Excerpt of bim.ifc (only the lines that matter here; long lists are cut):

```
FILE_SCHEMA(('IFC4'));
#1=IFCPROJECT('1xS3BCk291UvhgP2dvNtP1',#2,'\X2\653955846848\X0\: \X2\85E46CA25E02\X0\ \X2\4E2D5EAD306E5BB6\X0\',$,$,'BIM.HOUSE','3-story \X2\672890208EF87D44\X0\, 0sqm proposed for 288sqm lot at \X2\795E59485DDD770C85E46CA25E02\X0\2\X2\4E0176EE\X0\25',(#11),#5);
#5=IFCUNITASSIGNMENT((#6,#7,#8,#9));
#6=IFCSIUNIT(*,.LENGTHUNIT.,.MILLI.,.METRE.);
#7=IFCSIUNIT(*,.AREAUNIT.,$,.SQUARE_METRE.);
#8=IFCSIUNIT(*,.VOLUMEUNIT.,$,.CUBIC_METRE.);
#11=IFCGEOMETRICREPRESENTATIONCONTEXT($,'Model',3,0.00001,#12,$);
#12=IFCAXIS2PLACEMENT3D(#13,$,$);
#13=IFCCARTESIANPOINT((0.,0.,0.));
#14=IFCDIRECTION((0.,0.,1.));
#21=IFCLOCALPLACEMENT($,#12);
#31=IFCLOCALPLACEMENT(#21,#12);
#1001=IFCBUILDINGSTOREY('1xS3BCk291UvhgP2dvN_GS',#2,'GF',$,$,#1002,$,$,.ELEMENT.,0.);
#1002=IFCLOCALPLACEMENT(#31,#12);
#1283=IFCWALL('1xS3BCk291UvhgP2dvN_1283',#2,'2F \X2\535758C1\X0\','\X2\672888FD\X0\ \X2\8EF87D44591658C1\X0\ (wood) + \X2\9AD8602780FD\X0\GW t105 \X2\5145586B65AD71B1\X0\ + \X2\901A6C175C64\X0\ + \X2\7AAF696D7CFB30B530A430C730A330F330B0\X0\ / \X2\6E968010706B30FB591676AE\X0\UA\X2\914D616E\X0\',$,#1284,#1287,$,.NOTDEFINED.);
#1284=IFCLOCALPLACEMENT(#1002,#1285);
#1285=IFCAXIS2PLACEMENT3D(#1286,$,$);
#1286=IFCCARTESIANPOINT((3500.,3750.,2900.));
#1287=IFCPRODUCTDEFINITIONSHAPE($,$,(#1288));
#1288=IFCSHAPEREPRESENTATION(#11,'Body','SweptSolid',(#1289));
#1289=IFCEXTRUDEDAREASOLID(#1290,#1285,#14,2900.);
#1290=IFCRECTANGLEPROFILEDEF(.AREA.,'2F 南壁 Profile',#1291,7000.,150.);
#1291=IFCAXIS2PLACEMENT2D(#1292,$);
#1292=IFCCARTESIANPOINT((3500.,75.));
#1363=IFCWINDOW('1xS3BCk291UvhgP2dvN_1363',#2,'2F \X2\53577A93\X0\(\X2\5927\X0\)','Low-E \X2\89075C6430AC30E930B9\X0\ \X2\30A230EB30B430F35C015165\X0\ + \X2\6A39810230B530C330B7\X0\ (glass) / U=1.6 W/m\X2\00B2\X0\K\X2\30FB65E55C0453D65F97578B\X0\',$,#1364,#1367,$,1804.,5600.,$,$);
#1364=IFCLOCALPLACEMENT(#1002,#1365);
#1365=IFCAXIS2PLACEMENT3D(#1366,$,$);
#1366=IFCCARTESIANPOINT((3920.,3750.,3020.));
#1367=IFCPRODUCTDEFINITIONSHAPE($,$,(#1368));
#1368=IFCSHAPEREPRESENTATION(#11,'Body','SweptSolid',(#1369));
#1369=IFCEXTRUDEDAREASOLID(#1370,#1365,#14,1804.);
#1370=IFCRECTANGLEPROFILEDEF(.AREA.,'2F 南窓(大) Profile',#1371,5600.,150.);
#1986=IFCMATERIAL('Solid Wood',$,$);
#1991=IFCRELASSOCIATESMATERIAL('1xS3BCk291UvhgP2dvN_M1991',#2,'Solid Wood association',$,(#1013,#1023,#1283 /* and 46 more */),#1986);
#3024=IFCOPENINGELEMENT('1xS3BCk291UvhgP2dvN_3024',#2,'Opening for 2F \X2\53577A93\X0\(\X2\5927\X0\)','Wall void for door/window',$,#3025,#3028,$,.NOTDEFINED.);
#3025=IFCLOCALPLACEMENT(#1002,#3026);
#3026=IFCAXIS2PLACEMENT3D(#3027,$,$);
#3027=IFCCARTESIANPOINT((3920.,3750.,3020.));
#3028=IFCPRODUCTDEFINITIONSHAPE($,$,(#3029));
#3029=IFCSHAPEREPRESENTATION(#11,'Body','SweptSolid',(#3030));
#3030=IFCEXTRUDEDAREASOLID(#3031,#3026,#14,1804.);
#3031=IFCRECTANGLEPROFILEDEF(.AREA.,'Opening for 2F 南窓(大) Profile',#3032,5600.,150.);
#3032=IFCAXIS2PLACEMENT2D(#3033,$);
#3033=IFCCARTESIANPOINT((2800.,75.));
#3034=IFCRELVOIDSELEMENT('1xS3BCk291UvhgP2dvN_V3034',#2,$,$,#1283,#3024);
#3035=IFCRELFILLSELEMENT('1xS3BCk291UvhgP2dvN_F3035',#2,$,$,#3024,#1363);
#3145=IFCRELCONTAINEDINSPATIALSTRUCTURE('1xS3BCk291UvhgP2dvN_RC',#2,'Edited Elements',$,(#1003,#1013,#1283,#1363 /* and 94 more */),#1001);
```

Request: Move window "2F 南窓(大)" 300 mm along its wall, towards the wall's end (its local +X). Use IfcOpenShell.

```python
import ifcopenshell
import ifcopenshell.api.geometry
import ifcopenshell.util.placement

model = ifcopenshell.open("bim.ifc")

window = model.by_guid("1xS3BCk291UvhgP2dvN_1363")
opening = window.FillsVoids[0].RelatingOpeningElement
wall = opening.VoidsElements[0].RelatingBuildingElement

wall_matrix = ifcopenshell.util.placement.get_local_placement(wall.ObjectPlacement)
shift = wall_matrix[:3, 0] * 300.0
before = ifcopenshell.util.placement.get_local_placement(window.ObjectPlacement)[:3, 3].copy()

# The window is not placed relative to its opening, so move both.
for product in (opening, window):
    matrix = ifcopenshell.util.placement.get_local_placement(product.ObjectPlacement)
    matrix[:3, 3] += shift
    ifcopenshell.api.geometry.edit_object_placement(model, product=product, matrix=matrix, is_si=False)

after = ifcopenshell.util.placement.get_local_placement(window.ObjectPlacement)[:3, 3]
print("window moved by", (after - before).round(3) + 0.0)

model.write("bim_rev.ifc")
```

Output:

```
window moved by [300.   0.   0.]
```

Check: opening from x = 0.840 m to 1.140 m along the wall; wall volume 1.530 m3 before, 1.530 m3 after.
